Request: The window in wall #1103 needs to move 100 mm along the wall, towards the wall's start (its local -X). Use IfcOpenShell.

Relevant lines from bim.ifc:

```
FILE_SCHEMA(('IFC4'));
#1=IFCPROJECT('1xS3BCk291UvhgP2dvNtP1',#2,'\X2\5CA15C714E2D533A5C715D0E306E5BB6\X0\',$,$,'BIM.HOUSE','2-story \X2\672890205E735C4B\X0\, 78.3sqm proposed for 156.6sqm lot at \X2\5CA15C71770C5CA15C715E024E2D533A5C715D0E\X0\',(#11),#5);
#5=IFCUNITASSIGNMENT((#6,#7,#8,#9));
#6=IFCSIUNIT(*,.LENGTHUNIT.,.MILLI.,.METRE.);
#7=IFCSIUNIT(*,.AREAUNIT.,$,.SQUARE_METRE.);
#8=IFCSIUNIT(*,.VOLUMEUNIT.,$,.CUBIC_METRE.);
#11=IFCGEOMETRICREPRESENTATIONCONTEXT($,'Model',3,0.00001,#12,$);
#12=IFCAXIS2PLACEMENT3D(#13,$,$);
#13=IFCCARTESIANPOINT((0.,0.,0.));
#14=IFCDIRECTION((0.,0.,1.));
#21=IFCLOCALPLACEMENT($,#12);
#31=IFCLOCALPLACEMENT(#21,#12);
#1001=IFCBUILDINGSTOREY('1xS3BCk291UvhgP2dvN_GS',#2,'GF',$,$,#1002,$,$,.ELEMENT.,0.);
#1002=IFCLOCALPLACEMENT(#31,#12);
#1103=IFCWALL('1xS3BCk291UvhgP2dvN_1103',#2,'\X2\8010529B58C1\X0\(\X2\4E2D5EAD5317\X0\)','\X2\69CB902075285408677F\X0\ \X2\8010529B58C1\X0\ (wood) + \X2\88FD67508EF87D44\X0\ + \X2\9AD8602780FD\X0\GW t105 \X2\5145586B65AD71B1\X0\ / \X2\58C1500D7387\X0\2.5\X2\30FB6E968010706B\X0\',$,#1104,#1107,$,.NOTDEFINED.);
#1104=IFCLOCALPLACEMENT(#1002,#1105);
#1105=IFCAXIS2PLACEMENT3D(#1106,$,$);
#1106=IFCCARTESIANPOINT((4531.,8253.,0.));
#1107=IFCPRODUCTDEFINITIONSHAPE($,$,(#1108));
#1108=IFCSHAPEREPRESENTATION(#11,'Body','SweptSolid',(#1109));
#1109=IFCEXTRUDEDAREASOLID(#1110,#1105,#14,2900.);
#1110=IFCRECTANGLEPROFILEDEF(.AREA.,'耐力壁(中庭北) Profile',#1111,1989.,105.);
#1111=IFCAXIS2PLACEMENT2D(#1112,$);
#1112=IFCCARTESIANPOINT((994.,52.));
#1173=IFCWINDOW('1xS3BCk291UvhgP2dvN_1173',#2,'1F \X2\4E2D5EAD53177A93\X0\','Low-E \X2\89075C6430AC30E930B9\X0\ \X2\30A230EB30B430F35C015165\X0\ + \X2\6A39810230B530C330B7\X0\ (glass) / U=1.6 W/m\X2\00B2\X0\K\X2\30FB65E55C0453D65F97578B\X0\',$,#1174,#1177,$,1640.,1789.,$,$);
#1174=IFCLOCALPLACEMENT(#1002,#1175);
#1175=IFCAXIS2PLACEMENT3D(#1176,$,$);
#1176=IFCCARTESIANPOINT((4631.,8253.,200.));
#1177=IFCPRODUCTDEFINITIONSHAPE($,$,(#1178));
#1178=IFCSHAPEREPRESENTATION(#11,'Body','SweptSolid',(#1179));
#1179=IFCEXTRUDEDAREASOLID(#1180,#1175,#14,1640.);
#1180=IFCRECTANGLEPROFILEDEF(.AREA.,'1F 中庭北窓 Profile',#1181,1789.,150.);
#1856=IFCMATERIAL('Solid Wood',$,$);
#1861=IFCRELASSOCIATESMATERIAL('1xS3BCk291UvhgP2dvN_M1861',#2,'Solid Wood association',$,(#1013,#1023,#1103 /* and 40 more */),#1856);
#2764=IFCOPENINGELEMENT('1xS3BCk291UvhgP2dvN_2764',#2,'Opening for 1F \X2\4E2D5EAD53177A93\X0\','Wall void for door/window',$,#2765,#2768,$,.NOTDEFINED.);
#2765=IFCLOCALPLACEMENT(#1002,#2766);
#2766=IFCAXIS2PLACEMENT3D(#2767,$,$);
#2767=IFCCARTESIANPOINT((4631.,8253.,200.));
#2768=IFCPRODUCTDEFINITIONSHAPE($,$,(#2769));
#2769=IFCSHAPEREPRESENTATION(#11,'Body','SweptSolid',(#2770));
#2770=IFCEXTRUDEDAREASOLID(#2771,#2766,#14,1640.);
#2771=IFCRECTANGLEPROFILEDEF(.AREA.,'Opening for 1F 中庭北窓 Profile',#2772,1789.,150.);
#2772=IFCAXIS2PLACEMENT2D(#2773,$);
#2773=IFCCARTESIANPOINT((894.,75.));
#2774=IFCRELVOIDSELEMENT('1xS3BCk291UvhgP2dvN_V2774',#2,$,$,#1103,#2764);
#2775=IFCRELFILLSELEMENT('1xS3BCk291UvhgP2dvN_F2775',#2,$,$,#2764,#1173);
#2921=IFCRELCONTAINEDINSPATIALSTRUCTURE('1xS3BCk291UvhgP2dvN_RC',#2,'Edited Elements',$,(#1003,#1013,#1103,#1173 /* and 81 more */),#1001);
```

```python
import ifcopenshell
import ifcopenshell.api.geometry
import ifcopenshell.util.placement
import ifcopenshell.util.unit

model = ifcopenshell.open("bim.ifc")
unit_scale = ifcopenshell.util.unit.calculate_unit_scale(model)

window = model.by_guid("1xS3BCk291UvhgP2dvN_1173")
opening = window.FillsVoids[0].RelatingOpeningElement
wall = opening.VoidsElements[0].RelatingBuildingElement

wall_matrix = ifcopenshell.util.placement.get_local_placement(wall.ObjectPlacement)
shift = wall_matrix[:3, 0] * -0.1 / unit_scale
before = ifcopenshell.util.placement.get_local_placement(window.ObjectPlacement)[:3, 3].copy()

# The window is not placed relative to its opening, so move both.
for product in (opening, window):
    matrix = ifcopenshell.util.placement.get_local_placement(product.ObjectPlacement)
    matrix[:3, 3] += shift
    ifcopenshell.api.geometry.edit_object_placement(model, product=product, matrix=matrix, is_si=False)

after = ifcopenshell.util.placement.get_local_placement(window.ObjectPlacement)[:3, 3]
print("window moved by", (after - before).round(3) + 0.0)

model.write("bim_updated.ifc")
```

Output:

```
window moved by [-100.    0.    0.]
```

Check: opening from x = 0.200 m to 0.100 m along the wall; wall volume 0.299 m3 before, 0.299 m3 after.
